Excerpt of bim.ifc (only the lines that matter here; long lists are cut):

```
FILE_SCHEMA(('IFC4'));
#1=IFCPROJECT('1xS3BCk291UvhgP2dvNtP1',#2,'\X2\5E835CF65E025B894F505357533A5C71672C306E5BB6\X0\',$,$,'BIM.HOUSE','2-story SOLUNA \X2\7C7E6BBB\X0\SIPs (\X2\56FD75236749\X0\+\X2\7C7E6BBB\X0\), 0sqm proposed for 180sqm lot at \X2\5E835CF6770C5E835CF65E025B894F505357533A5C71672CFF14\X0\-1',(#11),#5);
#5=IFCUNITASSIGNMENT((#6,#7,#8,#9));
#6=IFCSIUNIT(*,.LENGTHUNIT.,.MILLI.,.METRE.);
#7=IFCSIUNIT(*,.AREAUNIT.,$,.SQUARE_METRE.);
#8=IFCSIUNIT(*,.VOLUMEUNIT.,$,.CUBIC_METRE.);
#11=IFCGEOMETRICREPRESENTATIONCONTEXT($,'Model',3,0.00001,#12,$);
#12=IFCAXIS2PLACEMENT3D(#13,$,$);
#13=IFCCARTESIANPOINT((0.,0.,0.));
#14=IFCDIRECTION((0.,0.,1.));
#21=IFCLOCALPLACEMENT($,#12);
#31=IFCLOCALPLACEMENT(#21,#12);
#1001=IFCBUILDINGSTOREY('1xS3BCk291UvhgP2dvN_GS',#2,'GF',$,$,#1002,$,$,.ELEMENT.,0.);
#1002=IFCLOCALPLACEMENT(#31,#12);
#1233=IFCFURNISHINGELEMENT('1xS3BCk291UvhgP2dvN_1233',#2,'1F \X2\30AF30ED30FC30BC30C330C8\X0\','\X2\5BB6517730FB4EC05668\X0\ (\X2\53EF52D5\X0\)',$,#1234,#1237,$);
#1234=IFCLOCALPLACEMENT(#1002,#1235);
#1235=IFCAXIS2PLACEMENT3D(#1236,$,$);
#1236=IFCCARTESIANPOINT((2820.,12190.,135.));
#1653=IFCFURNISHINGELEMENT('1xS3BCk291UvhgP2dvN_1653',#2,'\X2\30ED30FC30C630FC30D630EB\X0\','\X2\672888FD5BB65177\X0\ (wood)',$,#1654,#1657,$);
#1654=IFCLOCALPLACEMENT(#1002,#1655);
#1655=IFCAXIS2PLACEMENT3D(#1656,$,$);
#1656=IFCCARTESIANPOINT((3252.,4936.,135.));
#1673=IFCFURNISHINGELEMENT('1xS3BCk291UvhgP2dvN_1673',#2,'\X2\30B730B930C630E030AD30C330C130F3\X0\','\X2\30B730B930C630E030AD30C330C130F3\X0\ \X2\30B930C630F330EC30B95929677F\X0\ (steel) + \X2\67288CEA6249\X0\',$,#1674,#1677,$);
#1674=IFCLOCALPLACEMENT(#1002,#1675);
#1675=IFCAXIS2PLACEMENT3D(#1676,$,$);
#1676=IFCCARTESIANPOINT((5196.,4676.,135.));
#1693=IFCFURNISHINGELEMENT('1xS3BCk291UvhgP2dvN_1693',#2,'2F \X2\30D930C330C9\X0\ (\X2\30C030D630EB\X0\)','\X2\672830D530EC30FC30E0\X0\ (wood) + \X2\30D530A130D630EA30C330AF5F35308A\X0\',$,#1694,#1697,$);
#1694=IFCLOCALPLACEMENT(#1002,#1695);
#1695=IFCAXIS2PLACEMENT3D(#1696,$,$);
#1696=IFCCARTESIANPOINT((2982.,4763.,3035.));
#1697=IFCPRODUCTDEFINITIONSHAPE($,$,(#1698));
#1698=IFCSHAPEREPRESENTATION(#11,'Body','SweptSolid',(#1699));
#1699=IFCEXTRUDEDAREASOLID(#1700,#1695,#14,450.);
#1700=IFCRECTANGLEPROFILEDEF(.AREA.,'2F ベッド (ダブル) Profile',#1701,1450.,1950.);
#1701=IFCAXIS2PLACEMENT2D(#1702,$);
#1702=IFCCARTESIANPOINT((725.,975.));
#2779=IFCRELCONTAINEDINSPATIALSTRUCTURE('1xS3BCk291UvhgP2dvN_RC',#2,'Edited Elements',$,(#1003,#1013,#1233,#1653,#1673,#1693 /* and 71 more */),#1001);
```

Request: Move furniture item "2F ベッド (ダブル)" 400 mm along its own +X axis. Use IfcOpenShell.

```python
import ifcopenshell
import ifcopenshell.api.geometry
import ifcopenshell.util.placement
import ifcopenshell.util.unit

model = ifcopenshell.open("bim.ifc")
unit_scale = ifcopenshell.util.unit.calculate_unit_scale(model)

item = model.by_guid("1xS3BCk291UvhgP2dvN_1693")
matrix = ifcopenshell.util.placement.get_local_placement(item.ObjectPlacement)
matrix[:3, 3] += matrix[:3, 0] * 0.4 / unit_scale
ifcopenshell.api.geometry.edit_object_placement(model, product=item, matrix=matrix, is_si=False)

print(ifcopenshell.util.placement.get_local_placement(item.ObjectPlacement).round(3) + 0.0)

model.write("bim_edited.ifc")
```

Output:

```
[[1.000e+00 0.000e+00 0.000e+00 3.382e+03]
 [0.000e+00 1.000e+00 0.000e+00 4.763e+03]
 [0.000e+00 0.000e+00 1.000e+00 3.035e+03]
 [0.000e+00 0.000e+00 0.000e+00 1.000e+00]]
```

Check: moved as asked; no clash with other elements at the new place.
